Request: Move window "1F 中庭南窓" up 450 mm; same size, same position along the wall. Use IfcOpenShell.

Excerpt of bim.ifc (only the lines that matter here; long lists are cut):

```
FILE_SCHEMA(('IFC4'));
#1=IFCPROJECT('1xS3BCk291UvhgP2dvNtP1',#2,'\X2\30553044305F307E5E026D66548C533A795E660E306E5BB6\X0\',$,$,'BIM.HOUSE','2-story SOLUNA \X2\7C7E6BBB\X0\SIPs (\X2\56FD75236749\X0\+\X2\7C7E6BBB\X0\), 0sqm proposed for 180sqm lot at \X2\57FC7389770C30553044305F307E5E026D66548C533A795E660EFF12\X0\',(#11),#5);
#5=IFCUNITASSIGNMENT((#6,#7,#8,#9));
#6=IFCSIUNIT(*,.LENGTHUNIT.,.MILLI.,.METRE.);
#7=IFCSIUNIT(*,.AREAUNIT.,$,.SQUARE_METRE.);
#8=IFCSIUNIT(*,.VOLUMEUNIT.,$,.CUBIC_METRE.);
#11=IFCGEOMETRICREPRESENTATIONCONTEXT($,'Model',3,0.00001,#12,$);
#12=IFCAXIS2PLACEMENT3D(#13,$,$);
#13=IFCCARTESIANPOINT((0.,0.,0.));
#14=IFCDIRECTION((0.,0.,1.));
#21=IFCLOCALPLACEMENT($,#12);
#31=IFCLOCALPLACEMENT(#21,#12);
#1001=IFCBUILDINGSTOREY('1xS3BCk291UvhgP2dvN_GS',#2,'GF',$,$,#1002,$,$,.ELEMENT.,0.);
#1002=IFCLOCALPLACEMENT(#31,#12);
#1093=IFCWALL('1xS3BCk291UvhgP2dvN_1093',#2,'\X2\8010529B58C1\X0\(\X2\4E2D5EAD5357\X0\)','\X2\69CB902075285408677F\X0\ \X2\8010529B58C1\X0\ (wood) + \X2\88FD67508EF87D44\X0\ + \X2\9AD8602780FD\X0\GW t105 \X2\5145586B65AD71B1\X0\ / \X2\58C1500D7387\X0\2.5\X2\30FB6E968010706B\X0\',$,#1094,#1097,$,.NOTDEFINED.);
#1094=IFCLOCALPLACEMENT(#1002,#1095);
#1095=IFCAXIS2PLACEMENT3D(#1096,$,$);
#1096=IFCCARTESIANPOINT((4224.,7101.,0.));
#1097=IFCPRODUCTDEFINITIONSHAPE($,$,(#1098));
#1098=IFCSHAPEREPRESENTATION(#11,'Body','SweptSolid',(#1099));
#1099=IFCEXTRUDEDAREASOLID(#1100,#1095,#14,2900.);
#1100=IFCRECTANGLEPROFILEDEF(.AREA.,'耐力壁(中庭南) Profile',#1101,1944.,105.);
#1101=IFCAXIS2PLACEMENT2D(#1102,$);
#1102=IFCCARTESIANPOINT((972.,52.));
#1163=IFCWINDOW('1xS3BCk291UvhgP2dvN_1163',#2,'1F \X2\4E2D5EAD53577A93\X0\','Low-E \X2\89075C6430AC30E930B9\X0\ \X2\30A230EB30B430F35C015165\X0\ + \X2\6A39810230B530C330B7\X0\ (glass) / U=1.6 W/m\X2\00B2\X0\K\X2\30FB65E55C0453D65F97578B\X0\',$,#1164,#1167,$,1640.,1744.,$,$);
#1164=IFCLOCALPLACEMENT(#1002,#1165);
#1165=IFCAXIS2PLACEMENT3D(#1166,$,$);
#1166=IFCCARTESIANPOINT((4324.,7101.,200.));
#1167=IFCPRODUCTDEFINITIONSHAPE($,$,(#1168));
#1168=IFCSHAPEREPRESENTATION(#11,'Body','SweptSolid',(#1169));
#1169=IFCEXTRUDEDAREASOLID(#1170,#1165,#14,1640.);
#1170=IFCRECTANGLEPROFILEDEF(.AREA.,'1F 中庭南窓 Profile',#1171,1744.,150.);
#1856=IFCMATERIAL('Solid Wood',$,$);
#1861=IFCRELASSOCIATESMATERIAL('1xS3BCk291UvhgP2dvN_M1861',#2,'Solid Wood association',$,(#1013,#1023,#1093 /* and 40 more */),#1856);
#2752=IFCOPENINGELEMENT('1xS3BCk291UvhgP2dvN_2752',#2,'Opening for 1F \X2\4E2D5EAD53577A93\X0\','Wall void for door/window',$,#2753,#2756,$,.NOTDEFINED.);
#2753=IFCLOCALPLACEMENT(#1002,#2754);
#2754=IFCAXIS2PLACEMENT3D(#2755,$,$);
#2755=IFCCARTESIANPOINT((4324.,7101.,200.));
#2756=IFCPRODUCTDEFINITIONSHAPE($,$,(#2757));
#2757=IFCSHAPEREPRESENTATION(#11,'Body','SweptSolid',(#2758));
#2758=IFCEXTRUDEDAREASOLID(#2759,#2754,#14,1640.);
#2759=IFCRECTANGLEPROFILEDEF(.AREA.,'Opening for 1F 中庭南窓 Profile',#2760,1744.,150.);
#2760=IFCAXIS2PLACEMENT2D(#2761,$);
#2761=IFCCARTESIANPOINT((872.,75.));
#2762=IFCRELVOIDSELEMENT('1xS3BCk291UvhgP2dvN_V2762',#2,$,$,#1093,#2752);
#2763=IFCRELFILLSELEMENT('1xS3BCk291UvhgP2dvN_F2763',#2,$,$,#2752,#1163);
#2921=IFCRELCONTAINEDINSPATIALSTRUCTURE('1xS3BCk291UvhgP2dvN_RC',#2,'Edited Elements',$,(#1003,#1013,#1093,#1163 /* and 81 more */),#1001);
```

```python
import numpy as np
import ifcopenshell
import ifcopenshell.api.geometry
import ifcopenshell.util.placement
import ifcopenshell.util.unit

model = ifcopenshell.open("bim.ifc")
unit_scale = ifcopenshell.util.unit.calculate_unit_scale(model)

window = model.by_id(1163)
opening = window.FillsVoids[0].RelatingOpeningElement
dz = 450.0

shift = np.array([0.0, 0.0, dz])
# The window is not placed relative to its opening, so move both.
for product in (opening, window):
    matrix = ifcopenshell.util.placement.get_local_placement(product.ObjectPlacement)
    matrix[:3, 3] += shift
    ifcopenshell.api.geometry.edit_object_placement(model, product=product, matrix=matrix, is_si=False)

print(f"moved by {dz * unit_scale:+.3f} m")

model.write("bim-out.ifc")
```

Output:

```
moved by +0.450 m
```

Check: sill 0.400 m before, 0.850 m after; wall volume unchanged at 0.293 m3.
